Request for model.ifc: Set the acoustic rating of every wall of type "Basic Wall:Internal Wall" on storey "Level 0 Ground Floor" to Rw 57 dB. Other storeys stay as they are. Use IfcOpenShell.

First a look at what the model holds.

```python
import ifcopenshell
import ifcopenshell.util.element

model = ifcopenshell.open("model.ifc")
print(model.schema)
storey = next(s for s in model.by_type("IfcBuildingStorey") if s.Name == "Level 0 Ground Floor")
walls = [e for e in ifcopenshell.util.element.get_decomposition(storey) if e.is_a("IfcWall")]
seen = {}
for e in walls:
    element_type = ifcopenshell.util.element.get_type(e)
    key = (element_type.Name if element_type != e and element_type else None, ifcopenshell.util.element.get_pset(e, "Pset_WallCommon", "AcousticRating"))
    seen[key] = seen.get(key, 0) + 1
for (name, value), count in sorted(seen.items(), key=str):
    print(count, "x", name, "|", value)
```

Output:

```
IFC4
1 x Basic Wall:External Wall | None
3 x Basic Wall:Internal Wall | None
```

```python
import ifcopenshell
import ifcopenshell.api.pset
import ifcopenshell.util.element

model = ifcopenshell.open("model.ifc")

storey = next(s for s in model.by_type("IfcBuildingStorey") if s.Name == "Level 0 Ground Floor")
walls = [e for e in ifcopenshell.util.element.get_decomposition(storey) if e.is_a("IfcWall")]

count = 0
for e in walls:
    element_type = ifcopenshell.util.element.get_type(e)
    if element_type in (None, e) or element_type.Name != "Basic Wall:Internal Wall":
        continue
    # add_pset returns the element's existing set when there is one.
    pset = ifcopenshell.api.pset.add_pset(model, product=e, name="Pset_WallCommon")
    ifcopenshell.api.pset.edit_pset(model, pset=pset, properties={"AcousticRating": "Rw 57 dB"})
    count += 1

print(count, "walls updated")

model.write("model_updated.ifc")
```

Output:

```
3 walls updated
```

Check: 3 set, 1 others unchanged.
